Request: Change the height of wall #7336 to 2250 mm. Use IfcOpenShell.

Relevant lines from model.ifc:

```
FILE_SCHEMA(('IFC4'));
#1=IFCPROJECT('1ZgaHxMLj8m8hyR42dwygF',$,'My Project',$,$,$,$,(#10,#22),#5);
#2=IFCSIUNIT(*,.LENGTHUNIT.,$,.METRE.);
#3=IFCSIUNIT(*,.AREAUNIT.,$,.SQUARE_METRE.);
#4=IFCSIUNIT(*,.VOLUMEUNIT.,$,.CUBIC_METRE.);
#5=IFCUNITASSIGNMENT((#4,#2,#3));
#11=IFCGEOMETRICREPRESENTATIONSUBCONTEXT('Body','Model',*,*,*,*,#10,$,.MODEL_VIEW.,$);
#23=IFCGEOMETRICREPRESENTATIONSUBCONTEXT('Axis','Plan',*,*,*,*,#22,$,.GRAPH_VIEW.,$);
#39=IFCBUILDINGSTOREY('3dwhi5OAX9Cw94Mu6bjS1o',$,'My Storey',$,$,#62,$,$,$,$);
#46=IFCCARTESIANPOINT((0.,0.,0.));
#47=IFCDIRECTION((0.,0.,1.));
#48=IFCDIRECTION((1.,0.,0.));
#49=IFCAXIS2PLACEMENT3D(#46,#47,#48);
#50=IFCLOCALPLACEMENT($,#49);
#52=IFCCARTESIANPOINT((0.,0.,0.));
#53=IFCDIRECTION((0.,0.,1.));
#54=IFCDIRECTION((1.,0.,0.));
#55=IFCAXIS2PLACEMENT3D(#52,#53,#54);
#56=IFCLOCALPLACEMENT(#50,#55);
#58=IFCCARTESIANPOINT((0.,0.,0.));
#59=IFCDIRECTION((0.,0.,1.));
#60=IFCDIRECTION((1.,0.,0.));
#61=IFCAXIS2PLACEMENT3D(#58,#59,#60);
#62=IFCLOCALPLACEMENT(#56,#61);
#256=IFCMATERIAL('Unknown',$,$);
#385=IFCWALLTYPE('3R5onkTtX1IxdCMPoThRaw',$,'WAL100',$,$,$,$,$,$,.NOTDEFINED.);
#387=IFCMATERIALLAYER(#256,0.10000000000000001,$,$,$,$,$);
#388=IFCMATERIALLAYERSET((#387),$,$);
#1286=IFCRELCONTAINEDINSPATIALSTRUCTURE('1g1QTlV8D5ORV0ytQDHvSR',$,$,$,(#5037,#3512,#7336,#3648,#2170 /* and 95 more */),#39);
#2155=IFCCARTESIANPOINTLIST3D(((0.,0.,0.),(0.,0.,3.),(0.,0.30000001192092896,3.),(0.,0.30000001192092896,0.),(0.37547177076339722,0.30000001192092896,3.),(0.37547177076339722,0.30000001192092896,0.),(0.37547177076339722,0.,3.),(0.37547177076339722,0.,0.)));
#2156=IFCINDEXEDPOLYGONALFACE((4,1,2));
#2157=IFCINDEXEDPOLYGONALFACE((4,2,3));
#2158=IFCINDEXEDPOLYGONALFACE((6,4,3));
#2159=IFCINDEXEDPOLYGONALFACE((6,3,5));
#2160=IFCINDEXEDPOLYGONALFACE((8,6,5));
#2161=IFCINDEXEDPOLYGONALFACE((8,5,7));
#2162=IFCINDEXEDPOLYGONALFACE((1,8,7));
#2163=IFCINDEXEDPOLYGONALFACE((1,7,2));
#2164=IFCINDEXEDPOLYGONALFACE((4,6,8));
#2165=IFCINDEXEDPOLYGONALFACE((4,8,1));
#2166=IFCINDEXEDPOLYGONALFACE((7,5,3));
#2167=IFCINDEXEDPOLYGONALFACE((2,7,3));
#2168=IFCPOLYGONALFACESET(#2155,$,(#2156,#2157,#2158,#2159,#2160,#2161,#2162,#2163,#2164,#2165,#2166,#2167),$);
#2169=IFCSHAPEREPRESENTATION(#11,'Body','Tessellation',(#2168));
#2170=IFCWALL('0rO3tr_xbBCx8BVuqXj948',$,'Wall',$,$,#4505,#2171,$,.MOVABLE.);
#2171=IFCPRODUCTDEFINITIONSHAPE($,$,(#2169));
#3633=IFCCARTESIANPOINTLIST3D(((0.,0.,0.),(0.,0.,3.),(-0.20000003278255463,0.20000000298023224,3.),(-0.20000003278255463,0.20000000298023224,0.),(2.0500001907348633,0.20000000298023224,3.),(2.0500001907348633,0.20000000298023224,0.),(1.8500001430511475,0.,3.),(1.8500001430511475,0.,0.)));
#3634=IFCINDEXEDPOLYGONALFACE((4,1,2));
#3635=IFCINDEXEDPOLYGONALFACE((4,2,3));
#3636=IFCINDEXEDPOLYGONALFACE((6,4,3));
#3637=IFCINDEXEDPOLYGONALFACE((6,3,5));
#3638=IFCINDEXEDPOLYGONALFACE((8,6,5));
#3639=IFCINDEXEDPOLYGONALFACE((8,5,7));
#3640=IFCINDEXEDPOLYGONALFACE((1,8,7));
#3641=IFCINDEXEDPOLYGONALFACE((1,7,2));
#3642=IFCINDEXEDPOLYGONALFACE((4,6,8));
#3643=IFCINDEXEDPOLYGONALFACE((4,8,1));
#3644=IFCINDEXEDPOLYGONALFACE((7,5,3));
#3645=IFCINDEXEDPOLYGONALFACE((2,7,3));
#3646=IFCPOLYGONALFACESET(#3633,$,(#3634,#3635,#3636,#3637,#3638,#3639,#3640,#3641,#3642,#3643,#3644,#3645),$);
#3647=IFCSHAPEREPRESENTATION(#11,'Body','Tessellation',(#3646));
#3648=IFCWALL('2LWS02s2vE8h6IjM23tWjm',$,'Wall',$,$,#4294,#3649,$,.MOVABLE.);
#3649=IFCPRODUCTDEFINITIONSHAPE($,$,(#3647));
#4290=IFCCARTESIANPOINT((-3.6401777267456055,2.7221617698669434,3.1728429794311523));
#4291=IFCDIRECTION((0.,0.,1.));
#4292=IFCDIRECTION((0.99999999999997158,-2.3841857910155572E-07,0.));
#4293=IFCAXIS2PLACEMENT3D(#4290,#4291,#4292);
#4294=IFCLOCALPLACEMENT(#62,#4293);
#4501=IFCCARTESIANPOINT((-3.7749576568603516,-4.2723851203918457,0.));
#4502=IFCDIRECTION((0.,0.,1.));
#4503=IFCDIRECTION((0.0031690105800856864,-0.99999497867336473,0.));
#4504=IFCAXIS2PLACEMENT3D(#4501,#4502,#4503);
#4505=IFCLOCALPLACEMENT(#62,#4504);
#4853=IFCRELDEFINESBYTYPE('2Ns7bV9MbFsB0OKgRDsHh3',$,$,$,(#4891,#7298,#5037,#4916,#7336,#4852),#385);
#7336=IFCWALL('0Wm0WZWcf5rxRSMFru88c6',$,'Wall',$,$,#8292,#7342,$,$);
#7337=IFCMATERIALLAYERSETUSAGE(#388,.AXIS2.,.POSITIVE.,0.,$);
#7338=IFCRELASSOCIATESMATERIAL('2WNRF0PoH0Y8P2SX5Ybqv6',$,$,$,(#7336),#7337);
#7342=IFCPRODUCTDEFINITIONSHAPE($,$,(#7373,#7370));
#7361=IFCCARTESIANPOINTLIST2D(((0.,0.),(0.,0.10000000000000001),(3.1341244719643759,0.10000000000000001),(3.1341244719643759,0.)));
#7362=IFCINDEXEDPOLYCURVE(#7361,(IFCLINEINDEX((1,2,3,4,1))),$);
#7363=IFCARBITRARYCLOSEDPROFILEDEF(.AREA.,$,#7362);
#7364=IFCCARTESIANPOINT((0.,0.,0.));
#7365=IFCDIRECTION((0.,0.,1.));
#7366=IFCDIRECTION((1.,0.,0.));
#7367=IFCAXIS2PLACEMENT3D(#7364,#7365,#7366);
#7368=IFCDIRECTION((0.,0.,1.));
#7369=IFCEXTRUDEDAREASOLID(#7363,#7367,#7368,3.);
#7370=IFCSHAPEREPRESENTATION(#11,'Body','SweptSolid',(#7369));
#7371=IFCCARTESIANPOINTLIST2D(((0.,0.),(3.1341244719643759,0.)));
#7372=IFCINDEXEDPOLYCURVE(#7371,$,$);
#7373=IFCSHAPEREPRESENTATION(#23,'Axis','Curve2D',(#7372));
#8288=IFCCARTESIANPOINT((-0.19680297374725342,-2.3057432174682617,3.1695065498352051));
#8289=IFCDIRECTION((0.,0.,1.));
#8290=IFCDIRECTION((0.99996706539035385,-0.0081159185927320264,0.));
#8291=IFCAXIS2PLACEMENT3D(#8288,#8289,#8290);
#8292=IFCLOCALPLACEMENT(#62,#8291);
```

```python
import ifcopenshell
import ifcopenshell.geom
import ifcopenshell.util.representation
import ifcopenshell.util.shape

model = ifcopenshell.open("model.ifc")
settings = ifcopenshell.geom.settings()


def volume(element):
    """Net volume in cubic metres, openings subtracted."""
    shape = ifcopenshell.geom.create_shape(settings, element)
    return ifcopenshell.util.shape.get_volume(shape.geometry)


wall = model.by_id(7336)
before = volume(wall)

body = ifcopenshell.util.representation.get_representation(wall, "Model", "Body")
solid = body.Items[0]
old_height = solid.Depth
solid.Depth = 2.25
after = volume(wall)

print(f"height {old_height:g} -> {solid.Depth:g}, volume {before:.3f} -> {after:.3f} m3")

model.write("model_edited.ifc")
```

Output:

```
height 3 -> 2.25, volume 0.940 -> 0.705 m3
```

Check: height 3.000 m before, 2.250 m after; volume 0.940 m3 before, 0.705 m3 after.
